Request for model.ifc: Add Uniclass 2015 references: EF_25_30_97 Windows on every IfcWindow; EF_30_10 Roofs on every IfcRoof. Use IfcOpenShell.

First a look at what the model holds.

```python
import ifcopenshell

model = ifcopenshell.open("model.ifc")
print(model.schema)
print("classifications:", [c.Name for c in model.by_type("IfcClassification")])
for ifc_class in ("IfcDoor", "IfcRoof", "IfcStair", "IfcWall", "IfcWindow"):
    print(ifc_class, len(model.by_type(ifc_class)))
```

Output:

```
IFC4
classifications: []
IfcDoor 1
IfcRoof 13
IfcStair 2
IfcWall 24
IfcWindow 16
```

```python
import ifcopenshell
import ifcopenshell.api.classification

model = ifcopenshell.open("model.ifc")

system = ifcopenshell.api.classification.add_classification(model, classification="Uniclass 2015")

codes = {
    "IfcWindow": ("EF_25_30_97", "Windows"),
    "IfcRoof": ("EF_30_10", "Roofs"),
}
for ifc_class, (code, name) in codes.items():
    products = model.by_type(ifc_class)
    ifcopenshell.api.classification.add_reference(
        model, products=products, classification=system, identification=code, name=name
    )
    print(code, len(products))

model.write("model_rev.ifc")
```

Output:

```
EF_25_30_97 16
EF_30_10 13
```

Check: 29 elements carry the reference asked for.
